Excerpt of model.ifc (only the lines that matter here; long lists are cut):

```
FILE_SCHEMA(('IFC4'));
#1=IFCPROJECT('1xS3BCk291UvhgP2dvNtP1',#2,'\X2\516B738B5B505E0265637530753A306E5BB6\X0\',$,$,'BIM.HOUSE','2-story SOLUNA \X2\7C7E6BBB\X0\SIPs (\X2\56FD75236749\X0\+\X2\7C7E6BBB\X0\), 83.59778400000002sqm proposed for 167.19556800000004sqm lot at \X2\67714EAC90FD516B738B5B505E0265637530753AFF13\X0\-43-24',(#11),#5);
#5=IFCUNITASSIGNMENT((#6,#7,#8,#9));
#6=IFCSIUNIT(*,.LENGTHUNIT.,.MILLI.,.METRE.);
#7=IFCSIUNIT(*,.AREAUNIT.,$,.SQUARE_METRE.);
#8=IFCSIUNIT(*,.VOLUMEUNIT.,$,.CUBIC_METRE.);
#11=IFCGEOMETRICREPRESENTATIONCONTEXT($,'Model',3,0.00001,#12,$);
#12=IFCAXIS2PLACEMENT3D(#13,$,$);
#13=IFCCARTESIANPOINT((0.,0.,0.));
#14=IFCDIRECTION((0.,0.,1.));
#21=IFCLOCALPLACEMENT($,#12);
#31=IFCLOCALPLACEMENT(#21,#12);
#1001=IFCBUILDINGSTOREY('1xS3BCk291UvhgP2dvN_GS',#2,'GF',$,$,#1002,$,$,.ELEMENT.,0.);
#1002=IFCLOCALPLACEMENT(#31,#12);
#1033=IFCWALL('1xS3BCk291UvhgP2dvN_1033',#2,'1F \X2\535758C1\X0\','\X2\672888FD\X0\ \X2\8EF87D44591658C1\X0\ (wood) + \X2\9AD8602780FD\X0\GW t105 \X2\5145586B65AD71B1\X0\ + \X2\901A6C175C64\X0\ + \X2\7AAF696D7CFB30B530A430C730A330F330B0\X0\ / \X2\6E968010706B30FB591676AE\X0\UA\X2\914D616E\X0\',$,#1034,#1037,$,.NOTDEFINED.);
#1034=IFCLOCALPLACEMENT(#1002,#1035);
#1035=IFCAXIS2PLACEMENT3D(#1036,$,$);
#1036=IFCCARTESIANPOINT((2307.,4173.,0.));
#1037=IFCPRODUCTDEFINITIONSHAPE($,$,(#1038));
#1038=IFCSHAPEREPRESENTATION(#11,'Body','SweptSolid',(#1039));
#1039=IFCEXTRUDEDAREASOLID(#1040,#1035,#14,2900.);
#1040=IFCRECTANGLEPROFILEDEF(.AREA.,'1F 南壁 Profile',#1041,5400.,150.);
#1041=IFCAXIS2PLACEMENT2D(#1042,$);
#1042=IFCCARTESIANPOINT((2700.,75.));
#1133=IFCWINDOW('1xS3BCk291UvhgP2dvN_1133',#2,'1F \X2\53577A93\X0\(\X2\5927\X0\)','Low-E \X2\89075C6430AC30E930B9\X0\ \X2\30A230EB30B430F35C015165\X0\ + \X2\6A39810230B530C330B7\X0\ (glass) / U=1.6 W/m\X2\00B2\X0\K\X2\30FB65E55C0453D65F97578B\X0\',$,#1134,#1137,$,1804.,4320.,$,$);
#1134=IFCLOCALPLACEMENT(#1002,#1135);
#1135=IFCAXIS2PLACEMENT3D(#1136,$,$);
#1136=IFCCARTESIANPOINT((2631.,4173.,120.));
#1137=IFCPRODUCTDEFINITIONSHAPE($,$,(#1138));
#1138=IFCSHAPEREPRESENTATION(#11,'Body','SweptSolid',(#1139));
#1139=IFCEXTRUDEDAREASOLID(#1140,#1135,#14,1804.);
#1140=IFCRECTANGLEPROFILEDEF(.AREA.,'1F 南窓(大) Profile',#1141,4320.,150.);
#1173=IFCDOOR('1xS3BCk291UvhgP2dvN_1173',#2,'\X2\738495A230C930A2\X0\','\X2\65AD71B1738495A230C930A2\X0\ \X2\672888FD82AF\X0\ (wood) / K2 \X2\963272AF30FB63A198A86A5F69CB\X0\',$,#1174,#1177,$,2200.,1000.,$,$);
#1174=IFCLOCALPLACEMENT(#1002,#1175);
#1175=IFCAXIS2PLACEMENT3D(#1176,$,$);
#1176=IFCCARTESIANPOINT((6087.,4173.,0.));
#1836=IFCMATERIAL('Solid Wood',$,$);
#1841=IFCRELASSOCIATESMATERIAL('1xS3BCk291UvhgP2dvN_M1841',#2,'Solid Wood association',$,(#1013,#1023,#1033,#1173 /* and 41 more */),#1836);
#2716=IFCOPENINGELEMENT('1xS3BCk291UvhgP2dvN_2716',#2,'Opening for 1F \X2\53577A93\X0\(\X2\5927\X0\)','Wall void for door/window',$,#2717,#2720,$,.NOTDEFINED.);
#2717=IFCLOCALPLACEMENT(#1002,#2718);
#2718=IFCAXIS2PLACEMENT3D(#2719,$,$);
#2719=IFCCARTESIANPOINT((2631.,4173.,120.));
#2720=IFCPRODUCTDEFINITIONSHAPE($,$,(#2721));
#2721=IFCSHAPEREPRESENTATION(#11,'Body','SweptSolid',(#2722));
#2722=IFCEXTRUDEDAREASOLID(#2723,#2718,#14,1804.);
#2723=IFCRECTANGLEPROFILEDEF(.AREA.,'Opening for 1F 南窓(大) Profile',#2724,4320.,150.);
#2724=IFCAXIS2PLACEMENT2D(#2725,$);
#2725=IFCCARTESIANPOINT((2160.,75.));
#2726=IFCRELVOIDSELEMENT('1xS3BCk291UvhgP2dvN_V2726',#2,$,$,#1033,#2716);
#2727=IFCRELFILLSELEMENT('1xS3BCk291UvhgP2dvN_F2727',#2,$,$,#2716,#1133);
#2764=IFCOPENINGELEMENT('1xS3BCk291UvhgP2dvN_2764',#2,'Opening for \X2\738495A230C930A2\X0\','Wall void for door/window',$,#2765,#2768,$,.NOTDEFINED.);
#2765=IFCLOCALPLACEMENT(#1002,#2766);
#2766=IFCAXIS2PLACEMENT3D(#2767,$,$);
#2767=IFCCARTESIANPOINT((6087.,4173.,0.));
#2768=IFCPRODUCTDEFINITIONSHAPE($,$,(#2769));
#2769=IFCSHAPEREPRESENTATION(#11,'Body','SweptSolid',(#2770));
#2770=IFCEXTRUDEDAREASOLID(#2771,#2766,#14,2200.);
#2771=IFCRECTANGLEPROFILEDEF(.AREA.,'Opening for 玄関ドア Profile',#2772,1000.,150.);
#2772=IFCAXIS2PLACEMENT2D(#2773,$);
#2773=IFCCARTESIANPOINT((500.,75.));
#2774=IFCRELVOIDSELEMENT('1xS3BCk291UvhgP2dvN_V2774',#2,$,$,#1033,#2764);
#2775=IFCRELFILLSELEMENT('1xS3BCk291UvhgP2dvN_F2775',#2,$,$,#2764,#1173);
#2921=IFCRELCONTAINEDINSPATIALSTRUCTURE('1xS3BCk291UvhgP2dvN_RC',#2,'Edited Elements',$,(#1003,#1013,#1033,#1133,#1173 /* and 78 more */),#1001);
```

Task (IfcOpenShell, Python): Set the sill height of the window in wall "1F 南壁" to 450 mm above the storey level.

```python
import numpy as np
import ifcopenshell
import ifcopenshell.api.geometry
import ifcopenshell.geom
import ifcopenshell.util.element
import ifcopenshell.util.placement
import ifcopenshell.util.shape
import ifcopenshell.util.unit

model = ifcopenshell.open("model.ifc")
unit_scale = ifcopenshell.util.unit.calculate_unit_scale(model)

window = model.by_id(1133)
opening = window.FillsVoids[0].RelatingOpeningElement
storey = ifcopenshell.util.element.get_container(window, ifc_class="IfcBuildingStorey")
level = ifcopenshell.util.placement.get_local_placement(storey.ObjectPlacement)[2, 3]

# The opening's origin need not be at the sill, so measure its lowest point.
shape = ifcopenshell.geom.create_shape(ifcopenshell.geom.settings(), opening)
bottom = ifcopenshell.util.shape.get_shape_bottom_elevation(shape, shape.geometry) / unit_scale
dz = level + 0.45 / unit_scale - bottom

shift = np.array([0.0, 0.0, dz])
# The window is not placed relative to its opening, so move both.
for product in (opening, window):
    matrix = ifcopenshell.util.placement.get_local_placement(product.ObjectPlacement)
    matrix[:3, 3] += shift
    ifcopenshell.api.geometry.edit_object_placement(model, product=product, matrix=matrix, is_si=False)

print(f"moved by {dz * unit_scale:+.3f} m")

model.write("model_rev.ifc")
```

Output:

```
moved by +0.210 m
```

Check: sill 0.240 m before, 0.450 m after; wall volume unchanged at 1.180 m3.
